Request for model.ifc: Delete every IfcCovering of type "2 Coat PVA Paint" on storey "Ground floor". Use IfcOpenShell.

First a look at what the model holds.

```python
import ifcopenshell
import ifcopenshell.util.element

model = ifcopenshell.open("model.ifc")
print(model.schema)
storey = next(s for s in model.by_type("IfcBuildingStorey") if s.Name == "Ground floor")
coverings = [e for e in ifcopenshell.util.element.get_decomposition(storey) if e.is_a("IfcCovering")]
seen = {}
for e in coverings:
    element_type = ifcopenshell.util.element.get_type(e)
    name = element_type.Name if element_type not in (None, e) else None
    seen[name] = seen.get(name, 0) + 1
for name, count in sorted(seen.items(), key=str):
    print(count, "x", name)
```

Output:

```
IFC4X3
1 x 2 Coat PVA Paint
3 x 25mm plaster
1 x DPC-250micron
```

```python
import ifcopenshell
import ifcopenshell.api.root
import ifcopenshell.util.element

model = ifcopenshell.open("model.ifc")

storey = next(s for s in model.by_type("IfcBuildingStorey") if s.Name == "Ground floor")
coverings = [e for e in ifcopenshell.util.element.get_decomposition(storey) if e.is_a("IfcCovering")]
targets = [e for e in coverings if (t := ifcopenshell.util.element.get_type(e)) not in (None, e) and t.Name == "2 Coat PVA Paint"]

for e in targets:
    ifcopenshell.api.root.remove_product(model, product=e)
print(len(targets), "removed")

model.write("model_updated.ifc")
```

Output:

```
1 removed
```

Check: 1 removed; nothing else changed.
